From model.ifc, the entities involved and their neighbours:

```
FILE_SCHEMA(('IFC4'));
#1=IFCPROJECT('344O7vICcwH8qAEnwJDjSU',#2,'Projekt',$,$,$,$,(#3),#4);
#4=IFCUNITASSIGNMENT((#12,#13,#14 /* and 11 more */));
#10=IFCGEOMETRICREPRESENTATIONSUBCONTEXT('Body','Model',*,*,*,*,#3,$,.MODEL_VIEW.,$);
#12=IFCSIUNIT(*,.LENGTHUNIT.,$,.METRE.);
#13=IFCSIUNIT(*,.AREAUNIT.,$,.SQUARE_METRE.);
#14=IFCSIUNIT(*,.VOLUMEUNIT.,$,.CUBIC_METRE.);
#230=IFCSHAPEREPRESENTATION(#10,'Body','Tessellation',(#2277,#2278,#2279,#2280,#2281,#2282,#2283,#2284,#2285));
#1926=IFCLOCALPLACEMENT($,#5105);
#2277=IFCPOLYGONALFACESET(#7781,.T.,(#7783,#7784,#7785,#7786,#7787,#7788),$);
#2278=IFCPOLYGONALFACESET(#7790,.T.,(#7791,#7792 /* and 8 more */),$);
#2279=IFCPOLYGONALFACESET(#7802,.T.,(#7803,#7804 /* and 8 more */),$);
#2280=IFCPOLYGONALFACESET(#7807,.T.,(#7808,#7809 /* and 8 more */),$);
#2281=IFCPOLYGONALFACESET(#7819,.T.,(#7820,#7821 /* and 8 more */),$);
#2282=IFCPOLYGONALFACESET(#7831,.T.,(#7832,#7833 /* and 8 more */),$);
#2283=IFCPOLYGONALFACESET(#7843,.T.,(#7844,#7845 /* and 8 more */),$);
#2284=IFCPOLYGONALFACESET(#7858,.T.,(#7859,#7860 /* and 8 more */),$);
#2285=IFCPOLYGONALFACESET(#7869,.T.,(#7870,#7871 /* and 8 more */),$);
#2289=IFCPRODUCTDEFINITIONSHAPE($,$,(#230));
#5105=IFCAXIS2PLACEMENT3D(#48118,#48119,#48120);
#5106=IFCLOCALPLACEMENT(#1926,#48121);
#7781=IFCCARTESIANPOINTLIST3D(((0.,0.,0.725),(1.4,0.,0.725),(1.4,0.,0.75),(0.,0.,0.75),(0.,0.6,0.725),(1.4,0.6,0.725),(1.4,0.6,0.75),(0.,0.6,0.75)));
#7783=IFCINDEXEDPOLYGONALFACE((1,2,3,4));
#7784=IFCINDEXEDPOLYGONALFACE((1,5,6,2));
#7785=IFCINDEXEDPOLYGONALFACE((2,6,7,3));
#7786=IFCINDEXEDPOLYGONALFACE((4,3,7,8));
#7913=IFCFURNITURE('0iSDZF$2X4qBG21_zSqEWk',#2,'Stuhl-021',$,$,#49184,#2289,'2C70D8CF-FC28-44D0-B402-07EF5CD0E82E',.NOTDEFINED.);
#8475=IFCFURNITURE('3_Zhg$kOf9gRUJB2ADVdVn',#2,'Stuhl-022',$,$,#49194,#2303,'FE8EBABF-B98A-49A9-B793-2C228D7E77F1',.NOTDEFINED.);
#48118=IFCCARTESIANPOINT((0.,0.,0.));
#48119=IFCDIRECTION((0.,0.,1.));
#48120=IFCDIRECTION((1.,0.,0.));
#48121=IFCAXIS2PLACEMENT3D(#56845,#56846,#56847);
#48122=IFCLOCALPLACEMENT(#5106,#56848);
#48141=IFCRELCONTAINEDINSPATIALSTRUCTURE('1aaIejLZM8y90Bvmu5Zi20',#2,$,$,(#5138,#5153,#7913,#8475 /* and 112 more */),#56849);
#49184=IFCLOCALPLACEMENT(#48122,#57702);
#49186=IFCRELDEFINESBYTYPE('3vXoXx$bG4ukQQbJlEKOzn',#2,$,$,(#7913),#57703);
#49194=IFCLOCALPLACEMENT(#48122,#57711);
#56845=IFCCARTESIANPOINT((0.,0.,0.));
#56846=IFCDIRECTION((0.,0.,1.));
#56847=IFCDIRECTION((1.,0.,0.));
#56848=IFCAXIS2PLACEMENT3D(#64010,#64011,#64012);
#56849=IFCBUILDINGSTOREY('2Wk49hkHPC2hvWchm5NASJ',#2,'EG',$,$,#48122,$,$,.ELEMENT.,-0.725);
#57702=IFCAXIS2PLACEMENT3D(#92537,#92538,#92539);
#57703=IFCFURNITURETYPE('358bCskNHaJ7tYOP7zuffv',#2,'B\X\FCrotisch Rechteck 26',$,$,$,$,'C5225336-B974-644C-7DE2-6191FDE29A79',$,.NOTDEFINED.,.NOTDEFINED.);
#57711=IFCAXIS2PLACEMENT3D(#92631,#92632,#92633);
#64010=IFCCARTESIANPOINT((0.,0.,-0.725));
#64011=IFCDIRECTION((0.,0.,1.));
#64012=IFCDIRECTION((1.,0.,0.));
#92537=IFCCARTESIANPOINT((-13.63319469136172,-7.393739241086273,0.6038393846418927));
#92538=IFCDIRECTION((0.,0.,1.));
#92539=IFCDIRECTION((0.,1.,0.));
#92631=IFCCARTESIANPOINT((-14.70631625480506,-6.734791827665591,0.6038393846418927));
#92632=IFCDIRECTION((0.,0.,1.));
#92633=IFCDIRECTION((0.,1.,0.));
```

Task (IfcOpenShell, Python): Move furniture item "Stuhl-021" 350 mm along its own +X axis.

```python
import ifcopenshell
import ifcopenshell.api.geometry
import ifcopenshell.util.placement

model = ifcopenshell.open("model.ifc")

item = model.by_guid("0iSDZF$2X4qBG21_zSqEWk")
matrix = ifcopenshell.util.placement.get_local_placement(item.ObjectPlacement)
matrix[:3, 3] += matrix[:3, 0] * 0.35
ifcopenshell.api.geometry.edit_object_placement(model, product=item, matrix=matrix, is_si=False)

print(ifcopenshell.util.placement.get_local_placement(item.ObjectPlacement).round(3) + 0.0)

model.write("model_updated.ifc")
```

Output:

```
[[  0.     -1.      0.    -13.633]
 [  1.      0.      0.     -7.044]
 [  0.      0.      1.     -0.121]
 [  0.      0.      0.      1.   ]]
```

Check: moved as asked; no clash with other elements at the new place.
